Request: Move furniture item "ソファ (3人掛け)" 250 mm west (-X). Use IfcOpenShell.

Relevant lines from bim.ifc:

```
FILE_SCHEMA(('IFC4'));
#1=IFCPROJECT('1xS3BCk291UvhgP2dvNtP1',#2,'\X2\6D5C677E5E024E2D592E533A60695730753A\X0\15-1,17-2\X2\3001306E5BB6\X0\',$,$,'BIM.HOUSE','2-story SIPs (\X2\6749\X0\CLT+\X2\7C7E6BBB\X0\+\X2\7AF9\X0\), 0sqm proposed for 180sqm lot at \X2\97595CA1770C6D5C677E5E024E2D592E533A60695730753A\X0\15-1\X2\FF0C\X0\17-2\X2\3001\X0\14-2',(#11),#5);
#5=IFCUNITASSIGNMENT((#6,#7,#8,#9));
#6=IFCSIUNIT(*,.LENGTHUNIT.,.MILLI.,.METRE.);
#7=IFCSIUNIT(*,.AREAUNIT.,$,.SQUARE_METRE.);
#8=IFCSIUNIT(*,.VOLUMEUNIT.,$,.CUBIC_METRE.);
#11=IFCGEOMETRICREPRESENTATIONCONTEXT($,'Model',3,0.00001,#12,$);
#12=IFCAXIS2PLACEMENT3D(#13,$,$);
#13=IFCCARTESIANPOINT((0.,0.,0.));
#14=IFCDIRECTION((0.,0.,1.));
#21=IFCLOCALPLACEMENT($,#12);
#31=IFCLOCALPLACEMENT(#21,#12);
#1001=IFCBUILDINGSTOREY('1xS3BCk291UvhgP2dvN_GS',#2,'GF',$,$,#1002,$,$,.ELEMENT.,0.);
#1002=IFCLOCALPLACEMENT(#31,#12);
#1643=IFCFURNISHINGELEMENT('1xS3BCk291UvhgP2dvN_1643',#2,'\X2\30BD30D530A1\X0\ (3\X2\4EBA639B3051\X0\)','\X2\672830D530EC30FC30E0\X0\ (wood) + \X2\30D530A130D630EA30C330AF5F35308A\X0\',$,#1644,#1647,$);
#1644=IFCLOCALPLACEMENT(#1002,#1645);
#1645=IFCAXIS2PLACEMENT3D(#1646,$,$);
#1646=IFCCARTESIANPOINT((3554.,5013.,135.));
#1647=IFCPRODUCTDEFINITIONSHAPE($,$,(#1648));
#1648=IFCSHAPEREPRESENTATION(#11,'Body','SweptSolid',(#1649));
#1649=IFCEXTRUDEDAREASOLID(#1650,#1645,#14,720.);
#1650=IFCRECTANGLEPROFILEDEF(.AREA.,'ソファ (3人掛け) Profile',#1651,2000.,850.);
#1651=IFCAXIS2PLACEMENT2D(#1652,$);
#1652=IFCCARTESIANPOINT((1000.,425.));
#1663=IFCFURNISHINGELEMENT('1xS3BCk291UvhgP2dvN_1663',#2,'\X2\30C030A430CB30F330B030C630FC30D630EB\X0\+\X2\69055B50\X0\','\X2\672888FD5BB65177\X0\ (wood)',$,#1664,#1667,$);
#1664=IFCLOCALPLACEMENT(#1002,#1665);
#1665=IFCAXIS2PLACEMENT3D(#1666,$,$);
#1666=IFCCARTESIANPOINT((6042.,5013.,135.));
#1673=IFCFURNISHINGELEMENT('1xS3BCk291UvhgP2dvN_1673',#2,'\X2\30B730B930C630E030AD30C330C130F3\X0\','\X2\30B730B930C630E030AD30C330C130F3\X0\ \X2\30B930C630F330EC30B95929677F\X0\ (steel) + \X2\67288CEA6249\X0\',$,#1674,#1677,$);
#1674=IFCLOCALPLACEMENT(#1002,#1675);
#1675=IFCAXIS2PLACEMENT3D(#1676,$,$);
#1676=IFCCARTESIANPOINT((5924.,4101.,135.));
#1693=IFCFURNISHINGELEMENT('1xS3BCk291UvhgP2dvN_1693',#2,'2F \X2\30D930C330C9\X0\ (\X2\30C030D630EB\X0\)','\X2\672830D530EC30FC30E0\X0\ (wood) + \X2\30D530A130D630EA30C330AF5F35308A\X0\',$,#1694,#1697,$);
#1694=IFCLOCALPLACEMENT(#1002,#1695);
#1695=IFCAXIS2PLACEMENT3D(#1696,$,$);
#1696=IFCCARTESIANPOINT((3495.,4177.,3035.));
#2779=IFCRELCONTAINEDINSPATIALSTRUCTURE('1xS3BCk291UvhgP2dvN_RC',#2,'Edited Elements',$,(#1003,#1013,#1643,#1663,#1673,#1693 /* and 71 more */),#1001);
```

```python
import ifcopenshell
import ifcopenshell.api.geometry
import ifcopenshell.util.placement

model = ifcopenshell.open("bim.ifc")

item = model.by_guid("1xS3BCk291UvhgP2dvN_1643")
matrix = ifcopenshell.util.placement.get_local_placement(item.ObjectPlacement)
matrix[0, 3] -= 250.0
ifcopenshell.api.geometry.edit_object_placement(model, product=item, matrix=matrix, is_si=False)

print(ifcopenshell.util.placement.get_local_placement(item.ObjectPlacement).round(3) + 0.0)

model.write("bim_v2.ifc")
```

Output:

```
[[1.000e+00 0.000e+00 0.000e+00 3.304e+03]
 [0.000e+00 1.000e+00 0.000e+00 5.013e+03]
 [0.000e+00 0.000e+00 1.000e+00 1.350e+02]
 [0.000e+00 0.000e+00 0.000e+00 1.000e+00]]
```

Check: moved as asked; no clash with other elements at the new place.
